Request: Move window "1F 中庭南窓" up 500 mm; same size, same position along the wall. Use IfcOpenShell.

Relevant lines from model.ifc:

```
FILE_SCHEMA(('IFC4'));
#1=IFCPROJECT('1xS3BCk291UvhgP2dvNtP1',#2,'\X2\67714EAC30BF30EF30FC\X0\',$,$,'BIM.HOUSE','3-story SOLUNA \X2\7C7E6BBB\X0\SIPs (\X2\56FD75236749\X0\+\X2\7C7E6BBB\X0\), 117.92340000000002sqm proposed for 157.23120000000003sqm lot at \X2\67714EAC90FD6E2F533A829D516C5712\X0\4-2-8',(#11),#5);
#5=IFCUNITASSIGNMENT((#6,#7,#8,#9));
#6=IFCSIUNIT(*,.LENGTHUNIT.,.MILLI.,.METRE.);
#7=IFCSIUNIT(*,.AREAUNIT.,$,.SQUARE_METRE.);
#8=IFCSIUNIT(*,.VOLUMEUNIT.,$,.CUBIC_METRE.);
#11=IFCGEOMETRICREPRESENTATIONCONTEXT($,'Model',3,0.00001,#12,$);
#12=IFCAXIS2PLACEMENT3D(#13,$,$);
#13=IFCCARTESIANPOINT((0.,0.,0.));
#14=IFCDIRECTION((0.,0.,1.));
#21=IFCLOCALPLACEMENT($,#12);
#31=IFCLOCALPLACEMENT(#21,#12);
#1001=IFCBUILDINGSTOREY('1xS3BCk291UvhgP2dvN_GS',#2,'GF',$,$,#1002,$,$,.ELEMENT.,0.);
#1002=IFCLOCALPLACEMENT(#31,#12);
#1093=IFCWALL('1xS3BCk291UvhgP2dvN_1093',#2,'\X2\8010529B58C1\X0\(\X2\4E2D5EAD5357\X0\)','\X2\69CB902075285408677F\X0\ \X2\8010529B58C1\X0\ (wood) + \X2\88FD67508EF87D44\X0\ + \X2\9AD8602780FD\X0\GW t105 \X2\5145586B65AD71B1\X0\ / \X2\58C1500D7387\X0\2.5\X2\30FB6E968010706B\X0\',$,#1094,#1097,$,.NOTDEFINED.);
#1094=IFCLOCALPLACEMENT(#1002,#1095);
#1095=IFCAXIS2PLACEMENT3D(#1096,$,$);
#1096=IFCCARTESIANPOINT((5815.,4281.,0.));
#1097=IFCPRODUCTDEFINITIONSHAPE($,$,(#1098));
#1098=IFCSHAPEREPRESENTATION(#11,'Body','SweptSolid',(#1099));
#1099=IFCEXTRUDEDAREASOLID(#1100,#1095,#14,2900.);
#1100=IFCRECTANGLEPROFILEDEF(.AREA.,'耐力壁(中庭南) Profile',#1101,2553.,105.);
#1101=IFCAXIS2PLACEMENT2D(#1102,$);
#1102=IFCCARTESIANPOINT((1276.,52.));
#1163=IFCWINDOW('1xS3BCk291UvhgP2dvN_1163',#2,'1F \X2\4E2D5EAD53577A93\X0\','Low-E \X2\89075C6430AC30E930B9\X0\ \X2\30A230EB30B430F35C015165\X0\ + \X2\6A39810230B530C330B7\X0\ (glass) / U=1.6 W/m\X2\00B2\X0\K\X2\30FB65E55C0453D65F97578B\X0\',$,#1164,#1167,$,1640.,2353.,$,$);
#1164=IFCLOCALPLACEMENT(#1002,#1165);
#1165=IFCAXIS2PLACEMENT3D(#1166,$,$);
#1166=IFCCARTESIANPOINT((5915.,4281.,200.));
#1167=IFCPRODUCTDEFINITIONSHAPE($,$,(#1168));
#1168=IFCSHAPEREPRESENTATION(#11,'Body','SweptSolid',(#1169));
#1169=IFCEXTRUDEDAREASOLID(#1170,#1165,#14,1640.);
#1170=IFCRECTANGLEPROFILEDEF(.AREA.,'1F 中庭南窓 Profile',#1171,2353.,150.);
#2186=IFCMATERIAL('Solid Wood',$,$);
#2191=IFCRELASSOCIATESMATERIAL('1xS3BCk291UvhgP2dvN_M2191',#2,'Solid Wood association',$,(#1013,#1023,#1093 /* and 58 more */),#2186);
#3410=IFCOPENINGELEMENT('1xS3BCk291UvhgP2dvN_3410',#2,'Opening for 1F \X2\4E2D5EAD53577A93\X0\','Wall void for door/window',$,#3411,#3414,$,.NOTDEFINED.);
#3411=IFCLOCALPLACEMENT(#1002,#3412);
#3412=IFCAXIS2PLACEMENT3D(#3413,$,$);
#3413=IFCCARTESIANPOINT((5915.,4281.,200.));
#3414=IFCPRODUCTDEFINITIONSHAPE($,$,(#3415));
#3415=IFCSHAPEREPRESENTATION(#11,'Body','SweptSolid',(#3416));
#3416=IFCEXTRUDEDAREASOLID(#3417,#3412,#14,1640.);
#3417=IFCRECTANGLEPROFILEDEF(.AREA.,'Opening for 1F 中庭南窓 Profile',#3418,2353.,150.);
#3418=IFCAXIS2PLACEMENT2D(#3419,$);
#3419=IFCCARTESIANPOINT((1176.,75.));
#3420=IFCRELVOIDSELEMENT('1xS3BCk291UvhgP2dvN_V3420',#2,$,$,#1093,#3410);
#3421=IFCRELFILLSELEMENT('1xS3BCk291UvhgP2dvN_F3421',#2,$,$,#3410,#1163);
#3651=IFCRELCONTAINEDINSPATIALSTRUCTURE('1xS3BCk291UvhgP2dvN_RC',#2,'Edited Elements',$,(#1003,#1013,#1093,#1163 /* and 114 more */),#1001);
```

```python
import numpy as np
import ifcopenshell
import ifcopenshell.api.geometry
import ifcopenshell.util.placement
import ifcopenshell.util.unit

model = ifcopenshell.open("model.ifc")
unit_scale = ifcopenshell.util.unit.calculate_unit_scale(model)

window = model.by_id(1163)
opening = window.FillsVoids[0].RelatingOpeningElement
dz = 0.5 / unit_scale

shift = np.array([0.0, 0.0, dz])
# The window is not placed relative to its opening, so move both.
for product in (opening, window):
    matrix = ifcopenshell.util.placement.get_local_placement(product.ObjectPlacement)
    matrix[:3, 3] += shift
    ifcopenshell.api.geometry.edit_object_placement(model, product=product, matrix=matrix, is_si=False)

print(f"moved by {dz * unit_scale:+.3f} m")

model.write("model_rev.ifc")
```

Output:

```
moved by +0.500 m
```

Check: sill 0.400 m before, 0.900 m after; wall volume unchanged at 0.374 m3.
